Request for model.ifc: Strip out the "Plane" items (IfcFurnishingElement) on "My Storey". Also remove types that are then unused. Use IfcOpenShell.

First a look at what the model holds.

```python
import ifcopenshell
import ifcopenshell.util.element

model = ifcopenshell.open("model.ifc")
print(model.schema)
storey = next(s for s in model.by_type("IfcBuildingStorey") if s.Name == "My Storey")
furniture = [e for e in ifcopenshell.util.element.get_decomposition(storey) if e.is_a("IfcFurnishingElement")]
seen = {}
for e in furniture:
    element_type = ifcopenshell.util.element.get_type(e)
    name = element_type.Name if element_type not in (None, e) else None
    seen[name] = seen.get(name, 0) + 1
for name, count in sorted(seen.items(), key=str):
    print(count, "x", name)
```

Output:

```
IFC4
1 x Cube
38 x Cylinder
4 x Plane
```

```python
import ifcopenshell
import ifcopenshell.api.root
import ifcopenshell.util.element

model = ifcopenshell.open("model.ifc")

storey = next(s for s in model.by_type("IfcBuildingStorey") if s.Name == "My Storey")
furniture = [e for e in ifcopenshell.util.element.get_decomposition(storey) if e.is_a("IfcFurnishingElement")]
targets = [e for e in furniture if (t := ifcopenshell.util.element.get_type(e)) not in (None, e) and t.Name == "Plane"]
types = {ifcopenshell.util.element.get_type(e) for e in targets} - {None, *targets}

for e in targets:
    ifcopenshell.api.root.remove_product(model, product=e)
print(len(targets), "removed")

unused = [t for t in types if not ifcopenshell.util.element.get_types(t)]
for t in unused:
    ifcopenshell.api.root.remove_product(model, product=t)
print(len(unused), "unused types removed")

model.write("model_rev.ifc")
```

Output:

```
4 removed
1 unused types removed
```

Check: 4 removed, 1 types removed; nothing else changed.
